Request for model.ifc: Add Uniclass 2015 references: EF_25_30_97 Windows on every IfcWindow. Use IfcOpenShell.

First a look at what the model holds.

```python
import ifcopenshell

model = ifcopenshell.open("model.ifc")
print(model.schema)
print("classifications:", [c.Name for c in model.by_type("IfcClassification")])
for ifc_class in ("IfcDoor", "IfcRoof", "IfcStair", "IfcWall", "IfcWindow"):
    print(ifc_class, len(model.by_type(ifc_class)))
```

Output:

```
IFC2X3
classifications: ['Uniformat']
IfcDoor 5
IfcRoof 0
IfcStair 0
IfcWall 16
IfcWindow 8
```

```python
import ifcopenshell
import ifcopenshell.api.classification

model = ifcopenshell.open("model.ifc")

# IFC2X3 requires Source and Edition and has no link from the project to the system.
system = model.create_entity("IfcClassification", Source="NBS", Edition="2015", Name="Uniclass 2015")

codes = {
    "IfcWindow": ("EF_25_30_97", "Windows"),
}
for ifc_class, (code, name) in codes.items():
    products = model.by_type(ifc_class)
    ifcopenshell.api.classification.add_reference(
        model, products=products, classification=system, identification=code, name=name
    )
    print(code, len(products))

model.write("model_rev.ifc")
```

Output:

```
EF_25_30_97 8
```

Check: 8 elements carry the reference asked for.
